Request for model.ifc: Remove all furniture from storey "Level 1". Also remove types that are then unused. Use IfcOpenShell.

First a look at what the model holds.

```python
import ifcopenshell
import ifcopenshell.util.element

model = ifcopenshell.open("model.ifc")
print(model.schema)
storey = next(s for s in model.by_type("IfcBuildingStorey") if s.Name == "Level 1")
furniture = [e for e in ifcopenshell.util.element.get_decomposition(storey) if e.is_a("IfcFurnishingElement")]
seen = {}
for e in furniture:
    element_type = ifcopenshell.util.element.get_type(e)
    name = element_type.Name if element_type not in (None, e) else None
    seen[name] = seen.get(name, 0) + 1
for name, count in sorted(seen.items(), key=str):
    print(count, "x", name)
```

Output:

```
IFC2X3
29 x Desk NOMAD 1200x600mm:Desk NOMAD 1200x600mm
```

```python
import ifcopenshell
import ifcopenshell.api.root
import ifcopenshell.util.element

model = ifcopenshell.open("model.ifc")

storey = next(s for s in model.by_type("IfcBuildingStorey") if s.Name == "Level 1")
furniture = [e for e in ifcopenshell.util.element.get_decomposition(storey) if e.is_a("IfcFurnishingElement")]
types = {ifcopenshell.util.element.get_type(e) for e in furniture} - {None, *furniture}

for e in furniture:
    ifcopenshell.api.root.remove_product(model, product=e)
print(len(furniture), "removed")

unused = [t for t in types if not ifcopenshell.util.element.get_types(t)]
for t in unused:
    ifcopenshell.api.root.remove_product(model, product=t)
print(len(unused), "unused types removed")

model.write("model_v2.ifc")
```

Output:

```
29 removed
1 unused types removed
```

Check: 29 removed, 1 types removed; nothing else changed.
